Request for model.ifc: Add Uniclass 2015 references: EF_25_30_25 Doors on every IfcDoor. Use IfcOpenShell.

First a look at what the model holds.

```python
import ifcopenshell

model = ifcopenshell.open("model.ifc")
print(model.schema)
print("classifications:", [c.Name for c in model.by_type("IfcClassification")])
for ifc_class in ("IfcDoor", "IfcRoof", "IfcStair", "IfcWall", "IfcWindow"):
    print(ifc_class, len(model.by_type(ifc_class)))
```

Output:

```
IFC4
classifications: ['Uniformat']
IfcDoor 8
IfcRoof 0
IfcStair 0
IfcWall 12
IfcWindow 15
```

```python
import ifcopenshell
import ifcopenshell.api.classification

model = ifcopenshell.open("model.ifc")

system = ifcopenshell.api.classification.add_classification(model, classification="Uniclass 2015")

codes = {
    "IfcDoor": ("EF_25_30_25", "Doors"),
}
for ifc_class, (code, name) in codes.items():
    products = model.by_type(ifc_class)
    ifcopenshell.api.classification.add_reference(
        model, products=products, classification=system, identification=code, name=name
    )
    print(code, len(products))

model.write("model_v2.ifc")
```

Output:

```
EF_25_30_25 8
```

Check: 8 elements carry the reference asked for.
